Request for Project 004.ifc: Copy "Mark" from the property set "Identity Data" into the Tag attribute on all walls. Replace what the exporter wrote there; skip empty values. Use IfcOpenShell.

First a look at what the model holds.

```python
import ifcopenshell
import ifcopenshell.util.element

model = ifcopenshell.open("Project 004.ifc")
print(model.schema)
walls = model.by_type("IfcWall")
print(len(walls), "walls")
for e in walls[:8]:
    source = ifcopenshell.util.element.get_pset(e, "Identity Data", "Mark")
    target = e.Tag
    print(e.id(), repr(source), repr(target), sep=" | ")
```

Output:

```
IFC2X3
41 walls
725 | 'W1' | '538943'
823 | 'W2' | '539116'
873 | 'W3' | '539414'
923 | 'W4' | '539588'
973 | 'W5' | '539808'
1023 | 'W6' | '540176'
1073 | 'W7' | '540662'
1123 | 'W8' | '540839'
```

```python
import ifcopenshell
import ifcopenshell.util.element

model = ifcopenshell.open("Project 004.ifc")

count = 0
for e in model.by_type("IfcWall"):
    value = ifcopenshell.util.element.get_pset(e, "Identity Data", "Mark")
    current = e.Tag
    if not value or not value.strip() or current == value:
        continue
    e.Tag = value
    count += 1

print(count, "walls updated")

model.write("Project 004-out.ifc")
```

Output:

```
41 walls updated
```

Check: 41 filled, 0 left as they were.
